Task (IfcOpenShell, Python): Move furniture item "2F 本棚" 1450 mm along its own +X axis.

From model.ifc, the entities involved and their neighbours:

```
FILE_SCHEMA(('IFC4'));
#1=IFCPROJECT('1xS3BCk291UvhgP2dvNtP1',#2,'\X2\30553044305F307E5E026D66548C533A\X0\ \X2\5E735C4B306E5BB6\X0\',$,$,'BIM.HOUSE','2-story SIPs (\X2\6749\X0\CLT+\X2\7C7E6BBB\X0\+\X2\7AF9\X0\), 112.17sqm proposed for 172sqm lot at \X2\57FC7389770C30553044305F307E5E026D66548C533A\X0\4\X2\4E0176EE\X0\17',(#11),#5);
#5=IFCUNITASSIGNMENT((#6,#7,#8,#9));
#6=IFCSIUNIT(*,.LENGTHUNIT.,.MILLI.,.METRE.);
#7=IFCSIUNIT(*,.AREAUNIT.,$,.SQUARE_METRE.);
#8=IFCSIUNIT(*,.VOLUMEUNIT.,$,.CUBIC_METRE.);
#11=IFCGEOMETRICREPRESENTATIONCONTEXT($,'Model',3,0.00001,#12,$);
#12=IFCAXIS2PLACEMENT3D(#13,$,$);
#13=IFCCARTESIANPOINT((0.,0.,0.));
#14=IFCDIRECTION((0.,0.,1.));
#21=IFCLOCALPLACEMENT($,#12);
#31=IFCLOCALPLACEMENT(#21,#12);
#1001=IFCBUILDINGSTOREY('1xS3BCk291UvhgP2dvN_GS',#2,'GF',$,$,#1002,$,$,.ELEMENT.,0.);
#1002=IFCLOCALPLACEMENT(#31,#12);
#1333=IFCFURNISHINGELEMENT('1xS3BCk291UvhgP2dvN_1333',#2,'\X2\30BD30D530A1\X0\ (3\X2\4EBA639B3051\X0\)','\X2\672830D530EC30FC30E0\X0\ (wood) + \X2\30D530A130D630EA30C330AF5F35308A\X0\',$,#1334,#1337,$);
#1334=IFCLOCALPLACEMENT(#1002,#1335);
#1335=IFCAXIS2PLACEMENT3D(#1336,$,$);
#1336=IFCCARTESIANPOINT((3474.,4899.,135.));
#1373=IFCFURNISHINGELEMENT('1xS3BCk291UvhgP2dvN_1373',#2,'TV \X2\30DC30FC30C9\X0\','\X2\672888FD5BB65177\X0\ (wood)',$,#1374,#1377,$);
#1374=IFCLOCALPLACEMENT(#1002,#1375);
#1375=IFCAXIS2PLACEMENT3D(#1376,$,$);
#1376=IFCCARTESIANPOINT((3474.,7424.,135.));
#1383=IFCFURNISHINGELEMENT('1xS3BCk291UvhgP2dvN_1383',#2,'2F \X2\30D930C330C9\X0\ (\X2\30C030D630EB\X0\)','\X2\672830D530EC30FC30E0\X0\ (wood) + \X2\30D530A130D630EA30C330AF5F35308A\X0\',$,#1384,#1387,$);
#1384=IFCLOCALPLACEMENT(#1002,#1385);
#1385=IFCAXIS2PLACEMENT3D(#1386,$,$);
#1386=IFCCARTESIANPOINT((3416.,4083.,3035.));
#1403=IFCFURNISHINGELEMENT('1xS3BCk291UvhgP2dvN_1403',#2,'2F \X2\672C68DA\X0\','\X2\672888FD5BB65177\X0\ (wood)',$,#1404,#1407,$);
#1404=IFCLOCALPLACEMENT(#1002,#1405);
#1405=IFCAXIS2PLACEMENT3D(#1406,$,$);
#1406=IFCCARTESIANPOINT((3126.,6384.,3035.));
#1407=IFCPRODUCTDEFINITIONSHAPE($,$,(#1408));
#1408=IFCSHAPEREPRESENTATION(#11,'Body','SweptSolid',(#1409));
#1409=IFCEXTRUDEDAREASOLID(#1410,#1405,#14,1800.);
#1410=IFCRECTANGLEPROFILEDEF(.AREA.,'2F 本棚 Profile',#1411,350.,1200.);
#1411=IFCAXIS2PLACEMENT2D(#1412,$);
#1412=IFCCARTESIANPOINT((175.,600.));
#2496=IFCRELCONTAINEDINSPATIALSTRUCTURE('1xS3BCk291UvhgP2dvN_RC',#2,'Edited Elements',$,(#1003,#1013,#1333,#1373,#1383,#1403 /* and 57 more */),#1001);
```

```python
import ifcopenshell
import ifcopenshell.api.geometry
import ifcopenshell.util.placement

model = ifcopenshell.open("model.ifc")

item = model.by_id(1403)
matrix = ifcopenshell.util.placement.get_local_placement(item.ObjectPlacement)
matrix[:3, 3] += matrix[:3, 0] * 1450.0
ifcopenshell.api.geometry.edit_object_placement(model, product=item, matrix=matrix, is_si=False)

print(ifcopenshell.util.placement.get_local_placement(item.ObjectPlacement).round(3) + 0.0)

model.write("model_v2.ifc")
```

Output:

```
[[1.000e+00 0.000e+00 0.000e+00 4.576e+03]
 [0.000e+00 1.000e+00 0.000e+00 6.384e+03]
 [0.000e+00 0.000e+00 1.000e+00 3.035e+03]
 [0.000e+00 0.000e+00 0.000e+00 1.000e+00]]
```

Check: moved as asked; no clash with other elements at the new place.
